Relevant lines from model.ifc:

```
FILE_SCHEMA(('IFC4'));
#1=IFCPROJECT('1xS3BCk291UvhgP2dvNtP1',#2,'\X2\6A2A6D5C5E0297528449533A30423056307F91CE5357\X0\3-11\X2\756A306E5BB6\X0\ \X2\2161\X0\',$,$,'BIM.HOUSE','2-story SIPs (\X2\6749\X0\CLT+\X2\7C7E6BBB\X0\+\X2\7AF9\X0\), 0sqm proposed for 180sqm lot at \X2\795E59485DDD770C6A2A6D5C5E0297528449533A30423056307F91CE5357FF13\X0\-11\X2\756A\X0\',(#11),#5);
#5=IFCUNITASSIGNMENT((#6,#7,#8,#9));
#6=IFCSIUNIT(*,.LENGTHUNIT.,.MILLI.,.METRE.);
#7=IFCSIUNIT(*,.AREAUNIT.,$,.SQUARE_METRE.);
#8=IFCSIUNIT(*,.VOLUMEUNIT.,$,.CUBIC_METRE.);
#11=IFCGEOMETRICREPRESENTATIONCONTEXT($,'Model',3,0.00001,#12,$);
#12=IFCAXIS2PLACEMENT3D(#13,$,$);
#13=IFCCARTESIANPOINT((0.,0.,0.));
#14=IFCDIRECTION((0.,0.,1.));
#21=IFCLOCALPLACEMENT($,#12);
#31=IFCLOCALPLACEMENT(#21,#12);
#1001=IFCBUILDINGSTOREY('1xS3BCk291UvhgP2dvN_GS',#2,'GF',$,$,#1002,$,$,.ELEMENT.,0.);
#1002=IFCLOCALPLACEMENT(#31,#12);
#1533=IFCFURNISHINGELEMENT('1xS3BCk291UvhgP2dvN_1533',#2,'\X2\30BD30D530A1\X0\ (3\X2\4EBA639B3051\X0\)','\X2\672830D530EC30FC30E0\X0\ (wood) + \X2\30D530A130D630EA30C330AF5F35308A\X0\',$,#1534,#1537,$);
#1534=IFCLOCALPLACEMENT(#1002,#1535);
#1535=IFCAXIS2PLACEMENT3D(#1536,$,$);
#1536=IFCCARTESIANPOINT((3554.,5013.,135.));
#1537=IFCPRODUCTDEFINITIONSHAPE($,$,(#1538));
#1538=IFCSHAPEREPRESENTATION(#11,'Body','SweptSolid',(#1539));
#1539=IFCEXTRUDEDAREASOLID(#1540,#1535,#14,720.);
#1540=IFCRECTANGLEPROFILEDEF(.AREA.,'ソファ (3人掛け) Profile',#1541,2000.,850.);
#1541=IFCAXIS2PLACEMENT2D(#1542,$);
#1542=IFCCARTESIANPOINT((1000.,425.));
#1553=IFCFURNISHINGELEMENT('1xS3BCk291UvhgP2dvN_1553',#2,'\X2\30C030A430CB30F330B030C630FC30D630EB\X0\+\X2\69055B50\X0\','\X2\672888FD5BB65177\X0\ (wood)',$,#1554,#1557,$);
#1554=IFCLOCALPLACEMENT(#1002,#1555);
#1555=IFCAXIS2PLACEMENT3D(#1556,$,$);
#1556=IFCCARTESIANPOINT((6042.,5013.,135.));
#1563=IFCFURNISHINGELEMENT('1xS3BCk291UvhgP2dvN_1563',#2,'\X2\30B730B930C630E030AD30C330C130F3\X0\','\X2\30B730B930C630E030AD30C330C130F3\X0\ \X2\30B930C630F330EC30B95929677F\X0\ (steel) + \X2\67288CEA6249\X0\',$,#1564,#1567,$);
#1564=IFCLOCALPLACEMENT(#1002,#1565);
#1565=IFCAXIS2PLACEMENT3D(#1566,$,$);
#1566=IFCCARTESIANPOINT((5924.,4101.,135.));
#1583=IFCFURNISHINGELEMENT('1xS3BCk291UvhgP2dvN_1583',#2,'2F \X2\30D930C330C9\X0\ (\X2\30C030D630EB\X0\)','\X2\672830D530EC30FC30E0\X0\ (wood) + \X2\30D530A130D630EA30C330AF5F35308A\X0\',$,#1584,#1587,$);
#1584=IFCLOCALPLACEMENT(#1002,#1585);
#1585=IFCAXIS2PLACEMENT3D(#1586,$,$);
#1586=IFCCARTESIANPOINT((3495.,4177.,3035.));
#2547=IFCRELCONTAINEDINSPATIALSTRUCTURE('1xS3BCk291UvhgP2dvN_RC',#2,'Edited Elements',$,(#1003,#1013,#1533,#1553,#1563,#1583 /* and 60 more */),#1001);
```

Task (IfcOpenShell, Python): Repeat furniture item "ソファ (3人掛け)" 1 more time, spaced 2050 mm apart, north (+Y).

```python
import numpy as np
import ifcopenshell
import ifcopenshell.api.geometry
import ifcopenshell.api.root
import ifcopenshell.util.element
import ifcopenshell.util.placement

model = ifcopenshell.open("model.ifc")


def reuse_history(source, copy):
    """copy_class also copies each property set's owner history, people and application; keep the originals."""
    for rel in copy.IsDefinedBy:
        if rel.is_a("IfcRelDefinesByProperties") and (history := rel.RelatingPropertyDefinition.OwnerHistory):
            rel.RelatingPropertyDefinition.OwnerHistory = source.OwnerHistory
            ifcopenshell.util.element.remove_deep2(model, history)


source = model.by_guid("1xS3BCk291UvhgP2dvN_1533")
base = ifcopenshell.util.placement.get_local_placement(source.ObjectPlacement)
step = np.array([0.0, 1.0, 0.0]) * 2050.0

for i in range(1, 2):
    copy = ifcopenshell.api.root.copy_class(model, product=source)
    copy.Representation = ifcopenshell.util.element.copy_deep(
        model, source.Representation, exclude=["IfcGeometricRepresentationContext", "IfcRepresentationMap"]
    )
    reuse_history(source, copy)
    matrix = base.copy()
    matrix[:3, 3] += i * step
    print("added at", matrix[:3, 3].round(3) + 0.0)
    ifcopenshell.api.geometry.edit_object_placement(model, product=copy, matrix=matrix, is_si=False)

model.write("model_rev.ifc")
```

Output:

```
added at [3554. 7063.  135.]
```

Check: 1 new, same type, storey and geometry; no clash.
